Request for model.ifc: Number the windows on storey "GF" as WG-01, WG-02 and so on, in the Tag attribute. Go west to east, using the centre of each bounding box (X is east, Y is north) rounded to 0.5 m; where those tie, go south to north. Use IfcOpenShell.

First a look at what the model holds.

```python
import ifcopenshell
import ifcopenshell.util.element
import ifcopenshell.util.placement

model = ifcopenshell.open("model.ifc")
print(model.schema)
storey = next(s for s in model.by_type("IfcBuildingStorey") if s.Name == "GF")
windows = [e for e in ifcopenshell.util.element.get_decomposition(storey) if e.is_a("IfcWindow")]
for e in sorted(windows, key=lambda e: e.id()):
    origin = ifcopenshell.util.placement.get_local_placement(e.ObjectPlacement)[:3, 3]
    print(e.id(), e.Tag, e.Name, origin.round(2) + 0.0, sep=" | ")
```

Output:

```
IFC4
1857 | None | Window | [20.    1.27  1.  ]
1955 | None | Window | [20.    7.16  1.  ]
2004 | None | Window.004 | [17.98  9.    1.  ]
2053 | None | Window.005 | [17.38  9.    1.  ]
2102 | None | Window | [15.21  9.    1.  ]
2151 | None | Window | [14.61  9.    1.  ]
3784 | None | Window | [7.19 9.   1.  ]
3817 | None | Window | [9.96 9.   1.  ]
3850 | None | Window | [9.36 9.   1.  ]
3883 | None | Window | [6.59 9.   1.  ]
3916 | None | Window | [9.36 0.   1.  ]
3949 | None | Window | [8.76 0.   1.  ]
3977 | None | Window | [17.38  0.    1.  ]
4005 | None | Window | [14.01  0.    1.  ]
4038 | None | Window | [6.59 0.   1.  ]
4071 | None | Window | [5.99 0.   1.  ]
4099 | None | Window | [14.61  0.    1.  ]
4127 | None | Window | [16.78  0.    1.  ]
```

```python
import ifcopenshell
import ifcopenshell.geom
import ifcopenshell.util.element
import ifcopenshell.util.shape

model = ifcopenshell.open("model.ifc")
settings = ifcopenshell.geom.settings()
settings.set("use-world-coords", True)


def centre(element):
    shape = ifcopenshell.geom.create_shape(settings, element)
    return ifcopenshell.util.shape.get_bbox_centroid(shape.geometry)


storey = next(s for s in model.by_type("IfcBuildingStorey") if s.Name == "GF")
windows = [e for e in ifcopenshell.util.element.get_decomposition(storey) if e.is_a("IfcWindow")]

# Insertion points can sit at a corner or the storey origin, so sort by the geometry (in metres).
centres = {e: centre(e) for e in windows}
windows.sort(key=lambda e: (round(centres[e][0] / 0.5), centres[e][1]))

for i, e in enumerate(windows, start=1):
    number = f"WG-{i:02d}"
    e.Tag = number
    print(e.id(), number)

model.write("model_v2.ifc")
```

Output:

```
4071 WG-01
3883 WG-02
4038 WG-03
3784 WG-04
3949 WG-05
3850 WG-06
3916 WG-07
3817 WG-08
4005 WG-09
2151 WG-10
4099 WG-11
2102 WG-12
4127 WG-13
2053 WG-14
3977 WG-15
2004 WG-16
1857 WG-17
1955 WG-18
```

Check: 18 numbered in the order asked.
